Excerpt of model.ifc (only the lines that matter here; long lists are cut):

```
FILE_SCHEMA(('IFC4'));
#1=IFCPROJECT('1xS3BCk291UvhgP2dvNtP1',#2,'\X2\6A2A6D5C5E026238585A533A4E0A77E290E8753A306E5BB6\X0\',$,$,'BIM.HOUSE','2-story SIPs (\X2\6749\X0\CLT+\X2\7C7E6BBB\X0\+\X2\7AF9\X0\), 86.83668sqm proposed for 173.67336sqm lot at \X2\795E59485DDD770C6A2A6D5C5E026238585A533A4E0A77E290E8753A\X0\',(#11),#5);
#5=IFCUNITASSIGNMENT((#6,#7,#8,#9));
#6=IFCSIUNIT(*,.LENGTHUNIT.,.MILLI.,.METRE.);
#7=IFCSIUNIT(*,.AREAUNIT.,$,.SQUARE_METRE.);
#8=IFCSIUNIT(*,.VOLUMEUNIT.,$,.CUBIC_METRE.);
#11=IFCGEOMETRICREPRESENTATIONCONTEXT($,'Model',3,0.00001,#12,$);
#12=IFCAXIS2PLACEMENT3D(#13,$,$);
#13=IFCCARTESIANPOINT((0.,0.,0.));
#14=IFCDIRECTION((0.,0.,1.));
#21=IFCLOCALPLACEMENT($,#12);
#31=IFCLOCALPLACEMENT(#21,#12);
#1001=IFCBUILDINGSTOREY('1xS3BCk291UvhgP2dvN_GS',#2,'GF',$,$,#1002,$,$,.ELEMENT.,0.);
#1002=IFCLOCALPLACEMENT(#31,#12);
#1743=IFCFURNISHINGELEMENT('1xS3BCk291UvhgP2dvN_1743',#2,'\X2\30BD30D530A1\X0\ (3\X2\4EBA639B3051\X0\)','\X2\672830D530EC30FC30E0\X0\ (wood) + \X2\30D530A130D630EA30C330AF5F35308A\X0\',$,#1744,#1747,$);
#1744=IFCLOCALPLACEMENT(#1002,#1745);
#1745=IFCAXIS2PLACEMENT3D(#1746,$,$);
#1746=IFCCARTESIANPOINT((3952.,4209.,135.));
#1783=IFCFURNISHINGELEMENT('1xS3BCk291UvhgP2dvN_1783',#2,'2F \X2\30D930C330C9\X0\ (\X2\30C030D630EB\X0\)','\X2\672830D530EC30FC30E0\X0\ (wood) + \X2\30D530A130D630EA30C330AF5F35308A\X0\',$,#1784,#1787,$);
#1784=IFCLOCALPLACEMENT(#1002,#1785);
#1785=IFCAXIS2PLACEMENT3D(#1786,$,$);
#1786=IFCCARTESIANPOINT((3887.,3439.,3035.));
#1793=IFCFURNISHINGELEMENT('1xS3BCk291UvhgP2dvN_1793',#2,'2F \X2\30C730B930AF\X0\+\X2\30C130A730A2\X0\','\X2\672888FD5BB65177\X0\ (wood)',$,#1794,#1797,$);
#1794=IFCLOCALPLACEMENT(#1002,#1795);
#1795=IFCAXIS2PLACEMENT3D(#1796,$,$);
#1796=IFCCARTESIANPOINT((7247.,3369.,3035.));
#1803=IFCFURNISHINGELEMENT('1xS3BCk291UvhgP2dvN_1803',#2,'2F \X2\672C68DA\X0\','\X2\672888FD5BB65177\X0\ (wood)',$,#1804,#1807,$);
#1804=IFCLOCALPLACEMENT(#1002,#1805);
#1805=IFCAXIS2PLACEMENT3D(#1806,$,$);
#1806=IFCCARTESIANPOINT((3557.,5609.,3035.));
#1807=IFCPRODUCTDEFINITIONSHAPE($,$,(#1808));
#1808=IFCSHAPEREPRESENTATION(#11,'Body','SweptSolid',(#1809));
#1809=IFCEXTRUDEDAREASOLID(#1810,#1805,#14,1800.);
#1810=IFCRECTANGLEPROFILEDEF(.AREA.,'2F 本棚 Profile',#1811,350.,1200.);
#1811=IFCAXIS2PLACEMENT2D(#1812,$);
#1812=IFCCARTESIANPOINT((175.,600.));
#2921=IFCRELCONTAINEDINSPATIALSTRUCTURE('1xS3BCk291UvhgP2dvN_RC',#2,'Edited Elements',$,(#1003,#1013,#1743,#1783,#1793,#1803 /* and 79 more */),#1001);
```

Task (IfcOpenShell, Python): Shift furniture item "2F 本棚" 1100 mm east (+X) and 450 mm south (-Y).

```python
import ifcopenshell
import ifcopenshell.api.geometry
import ifcopenshell.util.placement

model = ifcopenshell.open("model.ifc")

item = model.by_guid("1xS3BCk291UvhgP2dvN_1803")
matrix = ifcopenshell.util.placement.get_local_placement(item.ObjectPlacement)
matrix[0, 3] += 1100.0
matrix[1, 3] -= 450.0
ifcopenshell.api.geometry.edit_object_placement(model, product=item, matrix=matrix, is_si=False)

print(ifcopenshell.util.placement.get_local_placement(item.ObjectPlacement).round(3) + 0.0)

model.write("model_rev.ifc")
```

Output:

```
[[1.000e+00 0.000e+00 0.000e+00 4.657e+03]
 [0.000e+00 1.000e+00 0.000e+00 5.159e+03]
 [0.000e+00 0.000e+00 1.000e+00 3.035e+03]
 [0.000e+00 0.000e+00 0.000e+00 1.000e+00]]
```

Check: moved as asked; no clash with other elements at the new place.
